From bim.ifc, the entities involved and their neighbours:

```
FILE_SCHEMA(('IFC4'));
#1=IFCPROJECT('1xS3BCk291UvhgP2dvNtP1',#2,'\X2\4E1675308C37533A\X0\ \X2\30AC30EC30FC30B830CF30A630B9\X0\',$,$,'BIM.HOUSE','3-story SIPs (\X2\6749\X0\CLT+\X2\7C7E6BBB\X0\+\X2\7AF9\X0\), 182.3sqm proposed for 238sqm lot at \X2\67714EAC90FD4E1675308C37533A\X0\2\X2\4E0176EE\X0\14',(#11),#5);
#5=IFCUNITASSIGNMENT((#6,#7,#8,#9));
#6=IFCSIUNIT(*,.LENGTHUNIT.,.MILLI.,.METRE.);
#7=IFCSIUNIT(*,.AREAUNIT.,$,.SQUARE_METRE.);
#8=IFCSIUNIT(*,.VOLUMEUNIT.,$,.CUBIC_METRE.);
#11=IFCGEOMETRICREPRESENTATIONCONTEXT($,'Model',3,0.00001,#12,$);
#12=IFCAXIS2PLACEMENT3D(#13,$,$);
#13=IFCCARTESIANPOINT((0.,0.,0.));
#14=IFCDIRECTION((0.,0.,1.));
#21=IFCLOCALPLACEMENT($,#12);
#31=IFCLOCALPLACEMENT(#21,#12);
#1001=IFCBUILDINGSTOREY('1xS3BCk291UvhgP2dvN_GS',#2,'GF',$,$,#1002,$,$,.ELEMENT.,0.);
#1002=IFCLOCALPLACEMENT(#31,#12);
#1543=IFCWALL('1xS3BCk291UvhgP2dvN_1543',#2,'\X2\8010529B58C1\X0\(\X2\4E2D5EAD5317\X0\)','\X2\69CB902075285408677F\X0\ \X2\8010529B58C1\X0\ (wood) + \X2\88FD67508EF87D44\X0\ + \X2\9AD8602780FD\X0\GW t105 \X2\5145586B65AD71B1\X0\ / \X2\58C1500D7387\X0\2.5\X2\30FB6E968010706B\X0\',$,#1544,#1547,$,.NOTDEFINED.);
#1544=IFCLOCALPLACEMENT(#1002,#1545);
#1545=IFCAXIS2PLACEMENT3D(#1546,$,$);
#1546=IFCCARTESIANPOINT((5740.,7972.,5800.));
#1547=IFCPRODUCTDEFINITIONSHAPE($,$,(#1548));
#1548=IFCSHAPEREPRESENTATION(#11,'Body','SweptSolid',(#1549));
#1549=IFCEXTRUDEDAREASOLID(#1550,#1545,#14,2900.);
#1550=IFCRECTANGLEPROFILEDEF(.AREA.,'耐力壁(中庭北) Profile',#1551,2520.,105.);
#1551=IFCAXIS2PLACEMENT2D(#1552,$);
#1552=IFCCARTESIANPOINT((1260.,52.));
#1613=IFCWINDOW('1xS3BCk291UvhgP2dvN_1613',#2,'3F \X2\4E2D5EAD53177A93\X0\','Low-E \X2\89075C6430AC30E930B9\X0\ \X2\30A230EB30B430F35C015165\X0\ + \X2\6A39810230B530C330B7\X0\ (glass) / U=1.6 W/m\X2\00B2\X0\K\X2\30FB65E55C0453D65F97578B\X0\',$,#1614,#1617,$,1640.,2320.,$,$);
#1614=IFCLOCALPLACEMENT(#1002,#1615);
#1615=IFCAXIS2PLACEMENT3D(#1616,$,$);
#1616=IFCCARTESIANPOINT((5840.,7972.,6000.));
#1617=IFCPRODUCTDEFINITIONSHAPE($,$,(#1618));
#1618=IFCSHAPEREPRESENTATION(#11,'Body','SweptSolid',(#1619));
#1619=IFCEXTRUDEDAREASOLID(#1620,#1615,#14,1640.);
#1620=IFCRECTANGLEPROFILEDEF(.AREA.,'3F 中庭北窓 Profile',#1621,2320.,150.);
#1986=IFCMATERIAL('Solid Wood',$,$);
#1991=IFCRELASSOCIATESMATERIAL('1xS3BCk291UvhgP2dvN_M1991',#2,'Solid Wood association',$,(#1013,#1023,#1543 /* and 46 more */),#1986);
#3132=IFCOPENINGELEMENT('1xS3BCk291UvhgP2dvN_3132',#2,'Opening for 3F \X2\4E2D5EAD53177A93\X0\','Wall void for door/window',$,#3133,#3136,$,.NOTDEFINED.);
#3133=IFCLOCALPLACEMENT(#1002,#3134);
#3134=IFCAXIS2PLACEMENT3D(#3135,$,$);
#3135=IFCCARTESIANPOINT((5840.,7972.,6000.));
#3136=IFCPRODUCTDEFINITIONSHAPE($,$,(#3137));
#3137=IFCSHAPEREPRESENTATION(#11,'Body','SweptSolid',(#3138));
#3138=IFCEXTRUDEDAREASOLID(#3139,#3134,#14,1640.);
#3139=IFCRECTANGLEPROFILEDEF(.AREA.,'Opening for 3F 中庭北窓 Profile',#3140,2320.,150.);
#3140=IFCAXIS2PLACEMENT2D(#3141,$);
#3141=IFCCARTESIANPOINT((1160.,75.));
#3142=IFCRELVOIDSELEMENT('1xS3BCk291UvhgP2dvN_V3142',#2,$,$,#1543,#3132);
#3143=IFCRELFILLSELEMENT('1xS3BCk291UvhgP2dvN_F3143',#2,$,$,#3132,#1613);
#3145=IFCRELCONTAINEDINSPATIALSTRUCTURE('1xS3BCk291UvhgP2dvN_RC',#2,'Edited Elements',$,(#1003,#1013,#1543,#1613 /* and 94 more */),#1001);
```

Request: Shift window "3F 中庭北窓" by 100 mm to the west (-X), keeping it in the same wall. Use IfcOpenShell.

```python
import ifcopenshell
import ifcopenshell.api.geometry
import ifcopenshell.util.placement
import ifcopenshell.util.unit

model = ifcopenshell.open("bim.ifc")
unit_scale = ifcopenshell.util.unit.calculate_unit_scale(model)

window = model.by_guid("1xS3BCk291UvhgP2dvN_1613")
opening = window.FillsVoids[0].RelatingOpeningElement
wall = opening.VoidsElements[0].RelatingBuildingElement

wall_matrix = ifcopenshell.util.placement.get_local_placement(wall.ObjectPlacement)
shift = wall_matrix[:3, 0] * -0.1 / unit_scale
before = ifcopenshell.util.placement.get_local_placement(window.ObjectPlacement)[:3, 3].copy()

# The window is not placed relative to its opening, so move both.
for product in (opening, window):
    matrix = ifcopenshell.util.placement.get_local_placement(product.ObjectPlacement)
    matrix[:3, 3] += shift
    ifcopenshell.api.geometry.edit_object_placement(model, product=product, matrix=matrix, is_si=False)

after = ifcopenshell.util.placement.get_local_placement(window.ObjectPlacement)[:3, 3]
print("window moved by", (after - before).round(3) + 0.0)

model.write("bim-out.ifc")
```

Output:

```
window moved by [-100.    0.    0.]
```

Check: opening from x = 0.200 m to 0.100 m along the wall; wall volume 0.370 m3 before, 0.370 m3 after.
